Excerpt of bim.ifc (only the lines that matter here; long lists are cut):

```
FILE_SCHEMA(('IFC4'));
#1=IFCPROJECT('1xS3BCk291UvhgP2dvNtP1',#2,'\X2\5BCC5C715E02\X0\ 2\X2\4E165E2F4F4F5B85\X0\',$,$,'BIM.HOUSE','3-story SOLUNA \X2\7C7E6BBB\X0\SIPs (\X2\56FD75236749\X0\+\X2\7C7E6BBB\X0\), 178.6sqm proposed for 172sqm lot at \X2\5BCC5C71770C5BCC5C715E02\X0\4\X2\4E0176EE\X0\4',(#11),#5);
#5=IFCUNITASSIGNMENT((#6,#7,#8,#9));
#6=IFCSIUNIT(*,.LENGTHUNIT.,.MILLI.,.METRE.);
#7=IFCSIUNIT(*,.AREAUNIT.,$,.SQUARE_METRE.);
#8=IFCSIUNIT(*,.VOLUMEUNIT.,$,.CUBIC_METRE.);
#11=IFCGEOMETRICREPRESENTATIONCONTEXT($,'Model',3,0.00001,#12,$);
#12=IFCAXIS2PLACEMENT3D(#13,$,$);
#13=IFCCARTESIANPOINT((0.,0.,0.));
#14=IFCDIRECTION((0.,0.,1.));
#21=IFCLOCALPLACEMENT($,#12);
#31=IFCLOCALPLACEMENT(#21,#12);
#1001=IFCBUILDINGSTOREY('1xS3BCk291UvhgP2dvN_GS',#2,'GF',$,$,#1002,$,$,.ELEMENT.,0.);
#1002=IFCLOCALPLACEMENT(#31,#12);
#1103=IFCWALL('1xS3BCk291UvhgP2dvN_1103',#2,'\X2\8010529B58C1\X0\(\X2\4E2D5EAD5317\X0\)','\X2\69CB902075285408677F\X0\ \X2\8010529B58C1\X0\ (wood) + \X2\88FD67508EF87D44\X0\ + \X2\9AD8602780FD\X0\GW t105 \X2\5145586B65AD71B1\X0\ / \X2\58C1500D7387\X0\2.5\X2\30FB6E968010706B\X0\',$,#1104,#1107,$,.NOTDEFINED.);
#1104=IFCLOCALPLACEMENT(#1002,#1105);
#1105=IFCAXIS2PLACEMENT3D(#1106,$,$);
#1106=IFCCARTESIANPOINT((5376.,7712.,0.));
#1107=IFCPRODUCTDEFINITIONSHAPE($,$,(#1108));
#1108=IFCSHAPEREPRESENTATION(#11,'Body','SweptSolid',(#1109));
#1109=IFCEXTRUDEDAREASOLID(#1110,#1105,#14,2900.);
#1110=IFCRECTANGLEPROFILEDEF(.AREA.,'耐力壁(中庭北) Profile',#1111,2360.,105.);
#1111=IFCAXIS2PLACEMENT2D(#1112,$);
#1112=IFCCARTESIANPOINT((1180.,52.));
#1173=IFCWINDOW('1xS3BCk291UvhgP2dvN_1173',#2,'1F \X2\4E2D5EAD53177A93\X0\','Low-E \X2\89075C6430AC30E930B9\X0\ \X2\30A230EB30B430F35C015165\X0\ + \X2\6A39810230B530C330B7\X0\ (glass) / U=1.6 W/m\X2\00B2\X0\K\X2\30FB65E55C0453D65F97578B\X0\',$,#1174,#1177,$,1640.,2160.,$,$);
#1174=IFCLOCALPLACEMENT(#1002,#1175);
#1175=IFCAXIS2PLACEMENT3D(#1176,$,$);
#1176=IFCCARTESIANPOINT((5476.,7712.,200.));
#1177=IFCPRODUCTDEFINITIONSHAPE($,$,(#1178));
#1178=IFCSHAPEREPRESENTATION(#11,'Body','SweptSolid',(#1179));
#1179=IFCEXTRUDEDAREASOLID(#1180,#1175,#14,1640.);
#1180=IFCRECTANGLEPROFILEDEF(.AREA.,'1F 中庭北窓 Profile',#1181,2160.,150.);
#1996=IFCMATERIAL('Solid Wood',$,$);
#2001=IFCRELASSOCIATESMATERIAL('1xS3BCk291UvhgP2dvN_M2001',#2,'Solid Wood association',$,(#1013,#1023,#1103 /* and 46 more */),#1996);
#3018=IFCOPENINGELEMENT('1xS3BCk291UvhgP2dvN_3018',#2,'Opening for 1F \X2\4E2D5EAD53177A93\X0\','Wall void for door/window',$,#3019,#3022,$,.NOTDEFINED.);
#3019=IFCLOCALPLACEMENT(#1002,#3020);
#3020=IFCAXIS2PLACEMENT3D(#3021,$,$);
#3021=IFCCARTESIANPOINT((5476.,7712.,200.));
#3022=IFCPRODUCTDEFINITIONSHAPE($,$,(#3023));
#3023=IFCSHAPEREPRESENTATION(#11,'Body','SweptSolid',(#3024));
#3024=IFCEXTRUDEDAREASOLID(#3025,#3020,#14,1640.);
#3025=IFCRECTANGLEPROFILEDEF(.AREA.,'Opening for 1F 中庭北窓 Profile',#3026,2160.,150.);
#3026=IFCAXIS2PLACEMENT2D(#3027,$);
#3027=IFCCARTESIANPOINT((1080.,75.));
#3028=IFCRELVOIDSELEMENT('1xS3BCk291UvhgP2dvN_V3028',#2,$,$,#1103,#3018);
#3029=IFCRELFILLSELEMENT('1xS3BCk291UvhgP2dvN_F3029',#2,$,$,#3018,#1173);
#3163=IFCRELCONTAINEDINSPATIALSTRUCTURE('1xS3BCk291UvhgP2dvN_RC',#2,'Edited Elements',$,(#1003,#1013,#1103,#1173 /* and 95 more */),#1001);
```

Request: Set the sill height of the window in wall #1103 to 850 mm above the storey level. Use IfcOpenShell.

```python
import numpy as np
import ifcopenshell
import ifcopenshell.api.geometry
import ifcopenshell.geom
import ifcopenshell.util.element
import ifcopenshell.util.placement
import ifcopenshell.util.shape
import ifcopenshell.util.unit

model = ifcopenshell.open("bim.ifc")
unit_scale = ifcopenshell.util.unit.calculate_unit_scale(model)

window = model.by_guid("1xS3BCk291UvhgP2dvN_1173")
opening = window.FillsVoids[0].RelatingOpeningElement
storey = ifcopenshell.util.element.get_container(window, ifc_class="IfcBuildingStorey")
level = ifcopenshell.util.placement.get_local_placement(storey.ObjectPlacement)[2, 3]

# The opening's origin need not be at the sill, so measure its lowest point.
shape = ifcopenshell.geom.create_shape(ifcopenshell.geom.settings(), opening)
bottom = ifcopenshell.util.shape.get_shape_bottom_elevation(shape, shape.geometry) / unit_scale
dz = level + 850.0 - bottom

shift = np.array([0.0, 0.0, dz])
# The window is not placed relative to its opening, so move both.
for product in (opening, window):
    matrix = ifcopenshell.util.placement.get_local_placement(product.ObjectPlacement)
    matrix[:3, 3] += shift
    ifcopenshell.api.geometry.edit_object_placement(model, product=product, matrix=matrix, is_si=False)

print(f"moved by {dz * unit_scale:+.3f} m")

model.write("bim_edited.ifc")
```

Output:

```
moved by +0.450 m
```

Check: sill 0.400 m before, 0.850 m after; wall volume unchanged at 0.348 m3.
